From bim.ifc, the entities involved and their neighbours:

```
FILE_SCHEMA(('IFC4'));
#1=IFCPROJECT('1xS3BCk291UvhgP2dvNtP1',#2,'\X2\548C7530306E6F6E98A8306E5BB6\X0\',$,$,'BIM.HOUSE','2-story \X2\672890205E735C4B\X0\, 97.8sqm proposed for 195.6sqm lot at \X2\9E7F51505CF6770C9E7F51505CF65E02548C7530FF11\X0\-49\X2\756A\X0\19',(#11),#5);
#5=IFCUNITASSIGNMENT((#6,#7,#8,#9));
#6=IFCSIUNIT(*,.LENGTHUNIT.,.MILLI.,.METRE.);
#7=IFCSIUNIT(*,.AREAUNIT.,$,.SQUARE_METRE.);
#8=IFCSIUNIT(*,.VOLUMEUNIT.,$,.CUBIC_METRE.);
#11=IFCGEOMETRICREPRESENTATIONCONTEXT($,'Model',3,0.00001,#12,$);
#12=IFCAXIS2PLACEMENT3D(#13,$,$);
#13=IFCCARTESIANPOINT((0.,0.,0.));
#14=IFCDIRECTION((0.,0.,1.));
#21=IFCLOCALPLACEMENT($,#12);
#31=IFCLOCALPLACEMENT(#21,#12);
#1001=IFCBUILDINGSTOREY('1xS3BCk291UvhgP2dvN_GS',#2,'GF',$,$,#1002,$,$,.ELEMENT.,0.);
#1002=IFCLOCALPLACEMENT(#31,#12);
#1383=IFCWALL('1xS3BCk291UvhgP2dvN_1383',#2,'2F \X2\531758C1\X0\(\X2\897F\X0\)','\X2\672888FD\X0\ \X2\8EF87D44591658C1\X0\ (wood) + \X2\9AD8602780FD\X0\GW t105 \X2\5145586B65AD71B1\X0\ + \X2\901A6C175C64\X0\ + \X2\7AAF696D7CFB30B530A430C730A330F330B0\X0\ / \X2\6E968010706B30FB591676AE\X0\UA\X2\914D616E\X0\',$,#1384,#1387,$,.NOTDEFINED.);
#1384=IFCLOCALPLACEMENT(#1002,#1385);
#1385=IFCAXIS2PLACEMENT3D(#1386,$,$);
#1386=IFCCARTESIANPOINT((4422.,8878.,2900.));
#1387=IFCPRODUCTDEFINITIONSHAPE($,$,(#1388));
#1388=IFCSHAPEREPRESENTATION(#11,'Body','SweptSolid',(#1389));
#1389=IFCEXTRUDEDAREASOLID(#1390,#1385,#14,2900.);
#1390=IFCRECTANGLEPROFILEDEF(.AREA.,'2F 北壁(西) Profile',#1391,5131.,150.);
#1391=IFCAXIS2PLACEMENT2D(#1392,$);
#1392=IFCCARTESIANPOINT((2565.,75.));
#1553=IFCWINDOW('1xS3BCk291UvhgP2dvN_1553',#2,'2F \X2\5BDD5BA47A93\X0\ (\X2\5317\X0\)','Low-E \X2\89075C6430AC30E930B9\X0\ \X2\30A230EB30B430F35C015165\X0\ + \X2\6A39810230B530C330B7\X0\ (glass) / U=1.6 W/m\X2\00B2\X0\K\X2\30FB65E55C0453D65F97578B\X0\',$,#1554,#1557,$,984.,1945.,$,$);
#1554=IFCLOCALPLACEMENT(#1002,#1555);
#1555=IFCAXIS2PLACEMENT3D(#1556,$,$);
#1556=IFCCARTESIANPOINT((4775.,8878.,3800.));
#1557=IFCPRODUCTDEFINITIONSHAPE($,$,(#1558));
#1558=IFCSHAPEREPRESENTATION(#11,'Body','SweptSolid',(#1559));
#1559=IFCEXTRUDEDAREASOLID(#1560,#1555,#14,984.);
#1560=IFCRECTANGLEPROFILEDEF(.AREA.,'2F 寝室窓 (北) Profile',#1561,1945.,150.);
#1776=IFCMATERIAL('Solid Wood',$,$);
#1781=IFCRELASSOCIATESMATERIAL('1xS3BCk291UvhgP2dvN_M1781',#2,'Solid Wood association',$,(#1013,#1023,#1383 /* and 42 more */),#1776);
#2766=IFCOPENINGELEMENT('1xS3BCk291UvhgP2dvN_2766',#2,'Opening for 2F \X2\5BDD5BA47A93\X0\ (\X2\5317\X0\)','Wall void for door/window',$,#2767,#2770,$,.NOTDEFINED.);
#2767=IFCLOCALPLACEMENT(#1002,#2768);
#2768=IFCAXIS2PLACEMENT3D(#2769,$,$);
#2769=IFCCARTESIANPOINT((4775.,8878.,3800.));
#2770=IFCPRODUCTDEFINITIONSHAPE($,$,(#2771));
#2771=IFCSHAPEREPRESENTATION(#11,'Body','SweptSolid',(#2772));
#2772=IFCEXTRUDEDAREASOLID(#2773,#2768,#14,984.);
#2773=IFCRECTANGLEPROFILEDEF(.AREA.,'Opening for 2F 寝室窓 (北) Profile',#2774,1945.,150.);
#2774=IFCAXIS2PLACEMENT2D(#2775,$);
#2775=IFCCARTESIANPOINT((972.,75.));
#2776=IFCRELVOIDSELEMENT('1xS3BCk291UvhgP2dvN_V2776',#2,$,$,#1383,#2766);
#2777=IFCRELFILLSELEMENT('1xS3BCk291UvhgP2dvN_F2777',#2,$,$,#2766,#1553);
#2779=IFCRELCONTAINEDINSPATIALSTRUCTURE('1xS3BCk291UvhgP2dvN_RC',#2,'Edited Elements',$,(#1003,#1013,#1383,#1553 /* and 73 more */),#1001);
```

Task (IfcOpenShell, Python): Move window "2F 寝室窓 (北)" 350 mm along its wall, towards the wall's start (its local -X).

```python
import ifcopenshell
import ifcopenshell.api.geometry
import ifcopenshell.util.placement
import ifcopenshell.util.unit

model = ifcopenshell.open("bim.ifc")
unit_scale = ifcopenshell.util.unit.calculate_unit_scale(model)

window = model.by_guid("1xS3BCk291UvhgP2dvN_1553")
opening = window.FillsVoids[0].RelatingOpeningElement
wall = opening.VoidsElements[0].RelatingBuildingElement

wall_matrix = ifcopenshell.util.placement.get_local_placement(wall.ObjectPlacement)
shift = wall_matrix[:3, 0] * -0.35 / unit_scale
before = ifcopenshell.util.placement.get_local_placement(window.ObjectPlacement)[:3, 3].copy()

# The window is not placed relative to its opening, so move both.
for product in (opening, window):
    matrix = ifcopenshell.util.placement.get_local_placement(product.ObjectPlacement)
    matrix[:3, 3] += shift
    ifcopenshell.api.geometry.edit_object_placement(model, product=product, matrix=matrix, is_si=False)

after = ifcopenshell.util.placement.get_local_placement(window.ObjectPlacement)[:3, 3]
print("window moved by", (after - before).round(3) + 0.0)

model.write("bim_edited.ifc")
```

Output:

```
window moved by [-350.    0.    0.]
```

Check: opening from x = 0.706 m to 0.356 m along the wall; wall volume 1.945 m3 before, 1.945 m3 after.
